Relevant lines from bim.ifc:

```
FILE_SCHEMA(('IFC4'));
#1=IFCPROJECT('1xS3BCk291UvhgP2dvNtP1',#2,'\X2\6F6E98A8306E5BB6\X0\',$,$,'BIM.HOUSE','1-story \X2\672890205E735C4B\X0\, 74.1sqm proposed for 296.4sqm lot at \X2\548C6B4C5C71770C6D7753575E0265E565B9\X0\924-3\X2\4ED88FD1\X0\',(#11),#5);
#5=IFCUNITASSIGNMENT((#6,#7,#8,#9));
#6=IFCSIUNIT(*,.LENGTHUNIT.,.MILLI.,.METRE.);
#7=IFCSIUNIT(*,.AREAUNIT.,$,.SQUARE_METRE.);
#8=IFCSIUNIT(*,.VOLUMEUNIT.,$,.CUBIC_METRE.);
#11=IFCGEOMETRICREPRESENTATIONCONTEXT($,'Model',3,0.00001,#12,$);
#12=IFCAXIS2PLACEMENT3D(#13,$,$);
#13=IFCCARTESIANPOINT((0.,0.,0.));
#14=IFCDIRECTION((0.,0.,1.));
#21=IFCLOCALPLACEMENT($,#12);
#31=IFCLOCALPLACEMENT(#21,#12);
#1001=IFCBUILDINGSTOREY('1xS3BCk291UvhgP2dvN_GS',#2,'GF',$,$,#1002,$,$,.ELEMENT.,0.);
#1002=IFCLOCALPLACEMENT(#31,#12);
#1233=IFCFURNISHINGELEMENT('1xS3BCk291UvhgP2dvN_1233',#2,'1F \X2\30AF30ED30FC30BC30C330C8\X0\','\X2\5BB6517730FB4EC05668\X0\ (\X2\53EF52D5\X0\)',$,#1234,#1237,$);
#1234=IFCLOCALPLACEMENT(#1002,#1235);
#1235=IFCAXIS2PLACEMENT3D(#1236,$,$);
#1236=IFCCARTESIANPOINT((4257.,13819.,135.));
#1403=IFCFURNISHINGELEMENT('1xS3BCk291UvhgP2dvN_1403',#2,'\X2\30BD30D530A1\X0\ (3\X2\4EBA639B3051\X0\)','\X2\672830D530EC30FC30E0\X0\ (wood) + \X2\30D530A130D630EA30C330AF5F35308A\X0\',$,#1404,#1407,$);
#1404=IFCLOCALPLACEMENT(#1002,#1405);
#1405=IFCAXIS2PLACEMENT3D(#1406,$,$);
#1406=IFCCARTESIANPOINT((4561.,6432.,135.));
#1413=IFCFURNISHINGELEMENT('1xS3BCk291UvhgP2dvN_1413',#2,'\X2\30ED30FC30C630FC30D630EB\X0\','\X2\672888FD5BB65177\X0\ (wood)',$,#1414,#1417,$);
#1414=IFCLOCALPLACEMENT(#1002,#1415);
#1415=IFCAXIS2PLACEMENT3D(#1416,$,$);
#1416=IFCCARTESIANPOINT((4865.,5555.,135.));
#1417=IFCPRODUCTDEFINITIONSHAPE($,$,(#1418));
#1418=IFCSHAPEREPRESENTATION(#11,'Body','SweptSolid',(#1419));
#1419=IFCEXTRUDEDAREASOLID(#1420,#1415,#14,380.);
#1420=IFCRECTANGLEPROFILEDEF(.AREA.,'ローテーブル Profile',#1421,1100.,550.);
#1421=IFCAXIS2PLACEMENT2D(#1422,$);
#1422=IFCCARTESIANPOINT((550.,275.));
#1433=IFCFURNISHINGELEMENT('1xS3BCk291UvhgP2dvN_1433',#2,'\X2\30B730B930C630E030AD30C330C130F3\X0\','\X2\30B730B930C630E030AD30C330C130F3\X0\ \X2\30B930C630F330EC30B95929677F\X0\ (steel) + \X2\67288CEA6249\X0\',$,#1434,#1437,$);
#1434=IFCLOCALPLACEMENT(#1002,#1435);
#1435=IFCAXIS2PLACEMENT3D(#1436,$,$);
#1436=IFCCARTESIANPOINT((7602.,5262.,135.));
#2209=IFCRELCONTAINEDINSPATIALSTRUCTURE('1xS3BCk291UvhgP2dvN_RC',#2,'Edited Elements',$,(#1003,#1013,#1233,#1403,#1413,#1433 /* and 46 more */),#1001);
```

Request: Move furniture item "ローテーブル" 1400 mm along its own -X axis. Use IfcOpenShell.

```python
import ifcopenshell
import ifcopenshell.api.geometry
import ifcopenshell.util.placement
import ifcopenshell.util.unit

model = ifcopenshell.open("bim.ifc")
unit_scale = ifcopenshell.util.unit.calculate_unit_scale(model)

item = model.by_guid("1xS3BCk291UvhgP2dvN_1413")
matrix = ifcopenshell.util.placement.get_local_placement(item.ObjectPlacement)
matrix[:3, 3] -= matrix[:3, 0] * 1.4 / unit_scale
ifcopenshell.api.geometry.edit_object_placement(model, product=item, matrix=matrix, is_si=False)

print(ifcopenshell.util.placement.get_local_placement(item.ObjectPlacement).round(3) + 0.0)

model.write("bim_edited.ifc")
```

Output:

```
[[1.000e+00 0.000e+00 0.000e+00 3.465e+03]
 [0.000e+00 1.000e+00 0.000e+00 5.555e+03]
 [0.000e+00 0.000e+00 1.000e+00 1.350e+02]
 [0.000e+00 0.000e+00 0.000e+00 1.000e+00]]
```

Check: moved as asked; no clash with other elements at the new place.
